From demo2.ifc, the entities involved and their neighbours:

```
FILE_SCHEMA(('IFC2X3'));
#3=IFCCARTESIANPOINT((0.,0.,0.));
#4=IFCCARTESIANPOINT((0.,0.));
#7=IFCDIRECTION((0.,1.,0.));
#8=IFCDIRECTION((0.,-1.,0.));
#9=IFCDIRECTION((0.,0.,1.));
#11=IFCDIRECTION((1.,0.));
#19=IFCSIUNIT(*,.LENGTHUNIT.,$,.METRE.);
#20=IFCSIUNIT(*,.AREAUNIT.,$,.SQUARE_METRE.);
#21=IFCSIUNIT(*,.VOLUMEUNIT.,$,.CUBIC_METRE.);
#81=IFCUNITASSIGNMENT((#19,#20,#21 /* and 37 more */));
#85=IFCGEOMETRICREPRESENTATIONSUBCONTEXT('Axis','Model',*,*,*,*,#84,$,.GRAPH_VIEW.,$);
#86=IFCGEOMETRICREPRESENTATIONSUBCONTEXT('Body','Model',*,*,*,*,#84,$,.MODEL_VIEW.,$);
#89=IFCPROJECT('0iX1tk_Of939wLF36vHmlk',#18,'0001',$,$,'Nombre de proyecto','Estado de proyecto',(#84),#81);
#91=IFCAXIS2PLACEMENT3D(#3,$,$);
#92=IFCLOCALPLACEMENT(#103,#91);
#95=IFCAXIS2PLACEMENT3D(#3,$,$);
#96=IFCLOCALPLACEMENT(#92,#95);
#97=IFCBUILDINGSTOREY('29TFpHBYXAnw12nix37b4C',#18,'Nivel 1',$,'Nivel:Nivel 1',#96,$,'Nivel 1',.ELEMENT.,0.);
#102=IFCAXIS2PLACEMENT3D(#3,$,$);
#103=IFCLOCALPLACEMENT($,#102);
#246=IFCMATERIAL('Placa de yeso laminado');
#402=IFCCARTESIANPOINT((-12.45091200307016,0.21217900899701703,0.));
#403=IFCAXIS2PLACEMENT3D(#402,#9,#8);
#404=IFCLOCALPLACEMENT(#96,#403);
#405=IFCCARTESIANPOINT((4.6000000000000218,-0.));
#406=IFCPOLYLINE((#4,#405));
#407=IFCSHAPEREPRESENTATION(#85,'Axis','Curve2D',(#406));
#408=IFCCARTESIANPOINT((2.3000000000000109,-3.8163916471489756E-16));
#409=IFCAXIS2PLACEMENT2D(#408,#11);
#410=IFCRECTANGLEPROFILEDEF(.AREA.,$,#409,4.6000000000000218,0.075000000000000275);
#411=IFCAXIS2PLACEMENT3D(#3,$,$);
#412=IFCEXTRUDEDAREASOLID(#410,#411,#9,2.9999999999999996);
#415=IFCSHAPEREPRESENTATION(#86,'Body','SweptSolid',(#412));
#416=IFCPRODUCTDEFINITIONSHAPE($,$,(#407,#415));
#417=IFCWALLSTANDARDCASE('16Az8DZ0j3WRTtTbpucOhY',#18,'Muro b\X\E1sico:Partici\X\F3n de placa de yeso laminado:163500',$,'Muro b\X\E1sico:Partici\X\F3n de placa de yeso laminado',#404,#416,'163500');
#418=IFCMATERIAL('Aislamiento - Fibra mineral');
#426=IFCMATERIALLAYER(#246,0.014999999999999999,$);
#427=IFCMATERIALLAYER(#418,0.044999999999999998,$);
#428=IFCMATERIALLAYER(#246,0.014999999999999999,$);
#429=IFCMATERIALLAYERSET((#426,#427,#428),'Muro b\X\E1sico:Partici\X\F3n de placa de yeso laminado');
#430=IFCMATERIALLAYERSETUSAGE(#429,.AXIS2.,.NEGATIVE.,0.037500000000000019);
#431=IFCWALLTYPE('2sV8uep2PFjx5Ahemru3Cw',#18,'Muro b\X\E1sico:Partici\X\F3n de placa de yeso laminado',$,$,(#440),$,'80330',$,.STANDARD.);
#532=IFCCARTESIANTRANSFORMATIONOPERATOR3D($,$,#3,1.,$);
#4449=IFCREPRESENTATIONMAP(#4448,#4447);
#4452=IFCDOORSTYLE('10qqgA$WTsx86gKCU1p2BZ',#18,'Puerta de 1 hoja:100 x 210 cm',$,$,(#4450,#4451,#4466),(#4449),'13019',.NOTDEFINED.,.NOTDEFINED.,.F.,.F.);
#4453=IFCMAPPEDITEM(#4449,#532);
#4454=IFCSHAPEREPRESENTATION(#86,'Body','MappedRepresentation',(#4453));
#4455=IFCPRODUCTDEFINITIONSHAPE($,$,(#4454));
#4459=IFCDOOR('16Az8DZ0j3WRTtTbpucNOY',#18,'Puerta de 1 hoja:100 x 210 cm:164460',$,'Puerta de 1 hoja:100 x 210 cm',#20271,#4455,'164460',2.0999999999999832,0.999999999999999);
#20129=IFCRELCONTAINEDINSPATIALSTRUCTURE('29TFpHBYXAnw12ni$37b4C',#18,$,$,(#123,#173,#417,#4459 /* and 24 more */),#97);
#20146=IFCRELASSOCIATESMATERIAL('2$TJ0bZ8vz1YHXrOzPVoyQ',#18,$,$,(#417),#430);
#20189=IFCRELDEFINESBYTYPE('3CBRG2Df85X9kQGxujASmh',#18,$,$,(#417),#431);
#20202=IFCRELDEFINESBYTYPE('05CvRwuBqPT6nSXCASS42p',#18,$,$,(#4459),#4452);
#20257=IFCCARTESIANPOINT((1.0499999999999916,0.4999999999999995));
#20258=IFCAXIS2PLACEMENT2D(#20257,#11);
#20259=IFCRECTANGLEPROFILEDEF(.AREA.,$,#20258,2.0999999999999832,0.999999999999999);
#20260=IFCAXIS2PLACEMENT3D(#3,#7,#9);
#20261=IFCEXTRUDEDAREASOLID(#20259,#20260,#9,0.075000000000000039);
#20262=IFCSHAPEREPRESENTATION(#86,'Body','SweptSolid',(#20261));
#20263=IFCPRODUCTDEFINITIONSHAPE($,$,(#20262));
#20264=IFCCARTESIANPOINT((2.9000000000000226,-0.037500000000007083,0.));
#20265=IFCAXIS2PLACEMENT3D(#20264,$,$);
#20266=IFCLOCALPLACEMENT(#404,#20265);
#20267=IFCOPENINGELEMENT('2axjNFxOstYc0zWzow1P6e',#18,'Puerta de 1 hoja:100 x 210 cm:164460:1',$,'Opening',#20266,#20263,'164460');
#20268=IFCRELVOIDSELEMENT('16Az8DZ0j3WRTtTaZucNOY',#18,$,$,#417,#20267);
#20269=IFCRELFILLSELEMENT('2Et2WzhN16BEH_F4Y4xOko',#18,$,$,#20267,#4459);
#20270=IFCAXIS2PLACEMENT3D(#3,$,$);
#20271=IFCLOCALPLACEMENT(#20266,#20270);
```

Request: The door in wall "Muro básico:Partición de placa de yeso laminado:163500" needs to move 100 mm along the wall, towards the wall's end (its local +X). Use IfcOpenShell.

```python
import ifcopenshell
import ifcopenshell.api.geometry
import ifcopenshell.util.placement
import ifcopenshell.util.unit

model = ifcopenshell.open("demo2.ifc")
unit_scale = ifcopenshell.util.unit.calculate_unit_scale(model)

door = model.by_guid("16Az8DZ0j3WRTtTbpucNOY")
opening = door.FillsVoids[0].RelatingOpeningElement
wall = opening.VoidsElements[0].RelatingBuildingElement

wall_matrix = ifcopenshell.util.placement.get_local_placement(wall.ObjectPlacement)
shift = wall_matrix[:3, 0] * 0.1 / unit_scale
before = ifcopenshell.util.placement.get_local_placement(door.ObjectPlacement)[:3, 3].copy()

# The door is placed relative to its opening, so it follows when the opening moves.
matrix = ifcopenshell.util.placement.get_local_placement(opening.ObjectPlacement)
matrix[:3, 3] += shift
ifcopenshell.api.geometry.edit_object_placement(
    model, product=opening, matrix=matrix, is_si=False, should_transform_children=True
)

after = ifcopenshell.util.placement.get_local_placement(door.ObjectPlacement)[:3, 3]
print("door moved by", (after - before).round(3) + 0.0)

model.write("demo2-out.ifc")
```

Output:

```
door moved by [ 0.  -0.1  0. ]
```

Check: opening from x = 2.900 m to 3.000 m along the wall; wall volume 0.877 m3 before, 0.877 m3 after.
